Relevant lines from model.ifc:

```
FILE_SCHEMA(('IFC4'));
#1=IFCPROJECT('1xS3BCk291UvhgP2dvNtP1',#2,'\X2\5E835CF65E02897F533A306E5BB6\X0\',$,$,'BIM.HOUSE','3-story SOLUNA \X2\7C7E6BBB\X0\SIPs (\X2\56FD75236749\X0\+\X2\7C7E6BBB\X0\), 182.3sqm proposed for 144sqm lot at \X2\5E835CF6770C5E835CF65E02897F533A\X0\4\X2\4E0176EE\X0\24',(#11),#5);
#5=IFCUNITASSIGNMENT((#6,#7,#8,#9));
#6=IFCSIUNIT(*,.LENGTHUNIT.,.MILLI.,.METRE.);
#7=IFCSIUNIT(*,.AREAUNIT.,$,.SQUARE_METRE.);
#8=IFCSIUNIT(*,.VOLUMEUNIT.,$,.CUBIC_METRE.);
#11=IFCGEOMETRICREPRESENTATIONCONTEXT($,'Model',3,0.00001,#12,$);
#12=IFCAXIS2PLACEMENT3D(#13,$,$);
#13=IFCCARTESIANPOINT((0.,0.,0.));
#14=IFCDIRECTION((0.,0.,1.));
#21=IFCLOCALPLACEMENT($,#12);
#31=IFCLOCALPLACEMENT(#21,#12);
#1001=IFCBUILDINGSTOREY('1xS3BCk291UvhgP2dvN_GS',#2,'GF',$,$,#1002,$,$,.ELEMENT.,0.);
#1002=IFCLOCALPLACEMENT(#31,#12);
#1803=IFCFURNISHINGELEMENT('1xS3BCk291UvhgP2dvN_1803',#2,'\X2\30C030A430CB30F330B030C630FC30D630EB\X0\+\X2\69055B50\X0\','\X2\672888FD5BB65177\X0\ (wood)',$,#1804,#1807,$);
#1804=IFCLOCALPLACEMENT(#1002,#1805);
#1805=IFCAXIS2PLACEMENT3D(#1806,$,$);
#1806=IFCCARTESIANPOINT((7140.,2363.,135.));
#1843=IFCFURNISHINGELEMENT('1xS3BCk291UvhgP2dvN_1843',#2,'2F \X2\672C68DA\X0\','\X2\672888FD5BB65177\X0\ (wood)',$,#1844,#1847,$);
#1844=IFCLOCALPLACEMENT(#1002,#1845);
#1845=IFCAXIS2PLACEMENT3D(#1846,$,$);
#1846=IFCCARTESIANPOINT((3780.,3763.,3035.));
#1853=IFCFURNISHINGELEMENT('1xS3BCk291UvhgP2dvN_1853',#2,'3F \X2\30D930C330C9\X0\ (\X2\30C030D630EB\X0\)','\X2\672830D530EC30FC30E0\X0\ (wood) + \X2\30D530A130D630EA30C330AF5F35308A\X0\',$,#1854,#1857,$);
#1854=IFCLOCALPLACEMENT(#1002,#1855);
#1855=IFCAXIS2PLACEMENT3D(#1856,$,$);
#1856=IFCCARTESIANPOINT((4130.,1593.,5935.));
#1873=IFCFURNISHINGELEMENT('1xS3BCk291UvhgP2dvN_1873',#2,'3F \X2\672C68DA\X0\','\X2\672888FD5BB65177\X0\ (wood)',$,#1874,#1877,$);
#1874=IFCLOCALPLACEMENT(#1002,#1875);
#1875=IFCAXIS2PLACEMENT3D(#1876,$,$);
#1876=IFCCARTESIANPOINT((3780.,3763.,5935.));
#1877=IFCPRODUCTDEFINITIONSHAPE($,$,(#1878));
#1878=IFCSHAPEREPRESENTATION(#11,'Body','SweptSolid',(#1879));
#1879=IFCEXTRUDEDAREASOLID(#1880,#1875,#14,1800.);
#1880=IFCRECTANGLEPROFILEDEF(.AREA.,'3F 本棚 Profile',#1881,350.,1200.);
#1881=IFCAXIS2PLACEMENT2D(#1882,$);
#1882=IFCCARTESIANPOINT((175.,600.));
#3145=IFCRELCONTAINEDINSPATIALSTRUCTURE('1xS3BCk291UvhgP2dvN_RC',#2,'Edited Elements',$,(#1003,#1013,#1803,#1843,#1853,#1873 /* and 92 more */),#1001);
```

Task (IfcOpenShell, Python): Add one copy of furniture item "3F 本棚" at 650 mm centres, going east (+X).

```python
import numpy as np
import ifcopenshell
import ifcopenshell.api.geometry
import ifcopenshell.api.root
import ifcopenshell.util.element
import ifcopenshell.util.placement

model = ifcopenshell.open("model.ifc")


def reuse_history(source, copy):
    """copy_class also copies each property set's owner history, people and application; keep the originals."""
    for rel in copy.IsDefinedBy:
        if rel.is_a("IfcRelDefinesByProperties") and (history := rel.RelatingPropertyDefinition.OwnerHistory):
            rel.RelatingPropertyDefinition.OwnerHistory = source.OwnerHistory
            ifcopenshell.util.element.remove_deep2(model, history)


source = model.by_guid("1xS3BCk291UvhgP2dvN_1873")
base = ifcopenshell.util.placement.get_local_placement(source.ObjectPlacement)
step = np.array([1.0, 0.0, 0.0]) * 650.0

for i in range(1, 2):
    copy = ifcopenshell.api.root.copy_class(model, product=source)
    copy.Representation = ifcopenshell.util.element.copy_deep(
        model, source.Representation, exclude=["IfcGeometricRepresentationContext", "IfcRepresentationMap"]
    )
    reuse_history(source, copy)
    matrix = base.copy()
    matrix[:3, 3] += i * step
    print("added at", matrix[:3, 3].round(3) + 0.0)
    ifcopenshell.api.geometry.edit_object_placement(model, product=copy, matrix=matrix, is_si=False)

model.write("model_v2.ifc")
```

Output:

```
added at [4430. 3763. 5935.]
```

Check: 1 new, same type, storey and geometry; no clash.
